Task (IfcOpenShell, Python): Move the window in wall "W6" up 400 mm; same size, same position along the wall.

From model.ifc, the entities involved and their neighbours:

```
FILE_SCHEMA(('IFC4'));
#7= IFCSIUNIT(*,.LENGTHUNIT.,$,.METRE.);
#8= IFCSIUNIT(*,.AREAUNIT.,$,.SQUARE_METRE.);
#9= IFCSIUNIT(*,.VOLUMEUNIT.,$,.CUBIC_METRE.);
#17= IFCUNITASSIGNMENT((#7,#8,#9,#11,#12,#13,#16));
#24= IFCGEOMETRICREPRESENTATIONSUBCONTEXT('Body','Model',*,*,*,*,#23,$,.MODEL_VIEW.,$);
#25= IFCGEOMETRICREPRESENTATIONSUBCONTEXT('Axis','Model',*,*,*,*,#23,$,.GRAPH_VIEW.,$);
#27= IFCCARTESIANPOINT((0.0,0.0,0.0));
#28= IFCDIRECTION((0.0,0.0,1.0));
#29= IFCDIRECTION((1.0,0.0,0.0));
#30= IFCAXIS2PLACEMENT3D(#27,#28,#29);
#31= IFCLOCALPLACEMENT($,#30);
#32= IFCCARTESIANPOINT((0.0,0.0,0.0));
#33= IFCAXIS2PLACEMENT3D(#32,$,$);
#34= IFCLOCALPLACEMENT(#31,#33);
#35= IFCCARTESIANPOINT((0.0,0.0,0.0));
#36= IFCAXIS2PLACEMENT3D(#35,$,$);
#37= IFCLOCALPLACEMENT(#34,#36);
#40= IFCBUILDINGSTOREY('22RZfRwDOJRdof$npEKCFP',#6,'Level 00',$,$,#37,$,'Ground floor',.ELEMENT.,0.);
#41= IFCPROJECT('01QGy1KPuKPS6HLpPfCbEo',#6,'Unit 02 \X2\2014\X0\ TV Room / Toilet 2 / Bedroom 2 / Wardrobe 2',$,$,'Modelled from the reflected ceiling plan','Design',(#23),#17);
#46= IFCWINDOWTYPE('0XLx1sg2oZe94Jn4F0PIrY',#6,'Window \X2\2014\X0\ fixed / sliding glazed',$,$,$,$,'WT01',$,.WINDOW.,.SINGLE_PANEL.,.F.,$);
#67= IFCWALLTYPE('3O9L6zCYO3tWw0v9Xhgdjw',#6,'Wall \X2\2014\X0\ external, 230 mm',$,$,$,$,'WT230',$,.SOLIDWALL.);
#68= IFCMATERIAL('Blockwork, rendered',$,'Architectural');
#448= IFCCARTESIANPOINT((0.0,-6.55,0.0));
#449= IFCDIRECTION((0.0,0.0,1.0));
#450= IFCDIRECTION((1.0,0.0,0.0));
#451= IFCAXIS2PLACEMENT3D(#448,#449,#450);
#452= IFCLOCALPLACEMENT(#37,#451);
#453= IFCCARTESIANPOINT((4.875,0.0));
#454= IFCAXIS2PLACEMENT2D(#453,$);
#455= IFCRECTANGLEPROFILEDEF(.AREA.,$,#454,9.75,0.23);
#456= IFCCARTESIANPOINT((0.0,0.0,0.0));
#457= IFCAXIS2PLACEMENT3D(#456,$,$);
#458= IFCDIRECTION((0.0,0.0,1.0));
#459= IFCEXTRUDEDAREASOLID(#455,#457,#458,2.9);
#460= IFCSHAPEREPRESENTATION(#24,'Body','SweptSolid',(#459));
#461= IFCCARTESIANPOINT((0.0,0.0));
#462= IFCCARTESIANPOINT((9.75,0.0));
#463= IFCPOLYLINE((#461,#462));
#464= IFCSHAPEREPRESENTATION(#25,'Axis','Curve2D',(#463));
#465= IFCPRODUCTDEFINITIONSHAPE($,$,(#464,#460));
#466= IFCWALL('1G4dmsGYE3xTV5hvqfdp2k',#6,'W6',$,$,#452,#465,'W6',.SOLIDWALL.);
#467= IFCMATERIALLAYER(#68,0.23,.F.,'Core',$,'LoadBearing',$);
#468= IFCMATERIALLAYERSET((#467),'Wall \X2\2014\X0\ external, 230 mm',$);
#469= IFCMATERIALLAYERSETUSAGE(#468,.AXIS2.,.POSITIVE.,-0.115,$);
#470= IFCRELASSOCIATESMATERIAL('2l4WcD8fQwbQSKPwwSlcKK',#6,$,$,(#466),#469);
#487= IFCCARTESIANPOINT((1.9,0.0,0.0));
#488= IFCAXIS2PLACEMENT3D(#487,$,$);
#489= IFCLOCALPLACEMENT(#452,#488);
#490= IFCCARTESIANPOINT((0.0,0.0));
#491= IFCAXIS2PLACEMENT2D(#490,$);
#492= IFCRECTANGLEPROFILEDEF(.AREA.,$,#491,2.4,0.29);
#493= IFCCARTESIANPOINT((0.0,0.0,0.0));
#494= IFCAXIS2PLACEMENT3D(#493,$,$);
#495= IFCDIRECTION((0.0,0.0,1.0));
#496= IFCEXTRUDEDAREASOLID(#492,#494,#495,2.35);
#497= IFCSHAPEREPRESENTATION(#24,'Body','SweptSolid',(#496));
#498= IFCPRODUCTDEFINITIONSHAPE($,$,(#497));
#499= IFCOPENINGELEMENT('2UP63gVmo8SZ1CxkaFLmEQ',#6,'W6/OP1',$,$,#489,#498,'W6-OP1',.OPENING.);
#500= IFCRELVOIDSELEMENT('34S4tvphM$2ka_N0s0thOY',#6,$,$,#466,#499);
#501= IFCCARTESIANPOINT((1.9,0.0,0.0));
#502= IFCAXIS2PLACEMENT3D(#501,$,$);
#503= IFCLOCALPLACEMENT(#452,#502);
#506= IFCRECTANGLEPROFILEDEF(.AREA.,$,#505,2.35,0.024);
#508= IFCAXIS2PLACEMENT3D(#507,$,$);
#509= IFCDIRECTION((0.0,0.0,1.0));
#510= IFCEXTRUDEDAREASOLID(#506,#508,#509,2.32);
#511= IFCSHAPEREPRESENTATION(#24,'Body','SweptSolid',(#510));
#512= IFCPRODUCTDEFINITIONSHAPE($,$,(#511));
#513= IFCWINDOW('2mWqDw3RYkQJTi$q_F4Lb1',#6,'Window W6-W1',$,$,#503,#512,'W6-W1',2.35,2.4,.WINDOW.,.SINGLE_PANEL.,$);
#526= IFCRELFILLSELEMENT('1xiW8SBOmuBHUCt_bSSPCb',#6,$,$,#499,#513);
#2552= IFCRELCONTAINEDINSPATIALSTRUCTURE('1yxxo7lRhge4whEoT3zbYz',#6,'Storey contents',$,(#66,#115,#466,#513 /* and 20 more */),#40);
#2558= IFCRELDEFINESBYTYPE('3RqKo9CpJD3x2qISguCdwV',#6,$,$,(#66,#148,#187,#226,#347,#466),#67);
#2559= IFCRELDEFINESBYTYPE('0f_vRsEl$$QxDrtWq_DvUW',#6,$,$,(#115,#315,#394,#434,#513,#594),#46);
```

```python
import numpy as np
import ifcopenshell
import ifcopenshell.api.geometry
import ifcopenshell.util.placement
import ifcopenshell.util.unit

model = ifcopenshell.open("model.ifc")
unit_scale = ifcopenshell.util.unit.calculate_unit_scale(model)

window = model.by_id(513)
opening = window.FillsVoids[0].RelatingOpeningElement
dz = 0.4 / unit_scale

shift = np.array([0.0, 0.0, dz])
# The window is not placed relative to its opening, so move both.
for product in (opening, window):
    matrix = ifcopenshell.util.placement.get_local_placement(product.ObjectPlacement)
    matrix[:3, 3] += shift
    ifcopenshell.api.geometry.edit_object_placement(model, product=product, matrix=matrix, is_si=False)

print(f"moved by {dz * unit_scale:+.3f} m")

model.write("model-out.ifc")
```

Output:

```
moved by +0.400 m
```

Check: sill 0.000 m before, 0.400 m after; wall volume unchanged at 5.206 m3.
